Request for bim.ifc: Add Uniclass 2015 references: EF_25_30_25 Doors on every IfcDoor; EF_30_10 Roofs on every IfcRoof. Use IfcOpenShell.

First a look at what the model holds.

```python
import ifcopenshell

model = ifcopenshell.open("bim.ifc")
print(model.schema)
print("classifications:", [c.Name for c in model.by_type("IfcClassification")])
for ifc_class in ("IfcDoor", "IfcRoof", "IfcStair", "IfcWall", "IfcWindow"):
    print(ifc_class, len(model.by_type(ifc_class)))
```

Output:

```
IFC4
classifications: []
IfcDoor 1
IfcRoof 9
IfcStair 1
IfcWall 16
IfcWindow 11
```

```python
import ifcopenshell
import ifcopenshell.api.classification

model = ifcopenshell.open("bim.ifc")

system = ifcopenshell.api.classification.add_classification(model, classification="Uniclass 2015")

codes = {
    "IfcDoor": ("EF_25_30_25", "Doors"),
    "IfcRoof": ("EF_30_10", "Roofs"),
}
for ifc_class, (code, name) in codes.items():
    products = model.by_type(ifc_class)
    ifcopenshell.api.classification.add_reference(
        model, products=products, classification=system, identification=code, name=name
    )
    print(code, len(products))

model.write("bim_edited.ifc")
```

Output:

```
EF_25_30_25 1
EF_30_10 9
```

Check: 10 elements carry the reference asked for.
